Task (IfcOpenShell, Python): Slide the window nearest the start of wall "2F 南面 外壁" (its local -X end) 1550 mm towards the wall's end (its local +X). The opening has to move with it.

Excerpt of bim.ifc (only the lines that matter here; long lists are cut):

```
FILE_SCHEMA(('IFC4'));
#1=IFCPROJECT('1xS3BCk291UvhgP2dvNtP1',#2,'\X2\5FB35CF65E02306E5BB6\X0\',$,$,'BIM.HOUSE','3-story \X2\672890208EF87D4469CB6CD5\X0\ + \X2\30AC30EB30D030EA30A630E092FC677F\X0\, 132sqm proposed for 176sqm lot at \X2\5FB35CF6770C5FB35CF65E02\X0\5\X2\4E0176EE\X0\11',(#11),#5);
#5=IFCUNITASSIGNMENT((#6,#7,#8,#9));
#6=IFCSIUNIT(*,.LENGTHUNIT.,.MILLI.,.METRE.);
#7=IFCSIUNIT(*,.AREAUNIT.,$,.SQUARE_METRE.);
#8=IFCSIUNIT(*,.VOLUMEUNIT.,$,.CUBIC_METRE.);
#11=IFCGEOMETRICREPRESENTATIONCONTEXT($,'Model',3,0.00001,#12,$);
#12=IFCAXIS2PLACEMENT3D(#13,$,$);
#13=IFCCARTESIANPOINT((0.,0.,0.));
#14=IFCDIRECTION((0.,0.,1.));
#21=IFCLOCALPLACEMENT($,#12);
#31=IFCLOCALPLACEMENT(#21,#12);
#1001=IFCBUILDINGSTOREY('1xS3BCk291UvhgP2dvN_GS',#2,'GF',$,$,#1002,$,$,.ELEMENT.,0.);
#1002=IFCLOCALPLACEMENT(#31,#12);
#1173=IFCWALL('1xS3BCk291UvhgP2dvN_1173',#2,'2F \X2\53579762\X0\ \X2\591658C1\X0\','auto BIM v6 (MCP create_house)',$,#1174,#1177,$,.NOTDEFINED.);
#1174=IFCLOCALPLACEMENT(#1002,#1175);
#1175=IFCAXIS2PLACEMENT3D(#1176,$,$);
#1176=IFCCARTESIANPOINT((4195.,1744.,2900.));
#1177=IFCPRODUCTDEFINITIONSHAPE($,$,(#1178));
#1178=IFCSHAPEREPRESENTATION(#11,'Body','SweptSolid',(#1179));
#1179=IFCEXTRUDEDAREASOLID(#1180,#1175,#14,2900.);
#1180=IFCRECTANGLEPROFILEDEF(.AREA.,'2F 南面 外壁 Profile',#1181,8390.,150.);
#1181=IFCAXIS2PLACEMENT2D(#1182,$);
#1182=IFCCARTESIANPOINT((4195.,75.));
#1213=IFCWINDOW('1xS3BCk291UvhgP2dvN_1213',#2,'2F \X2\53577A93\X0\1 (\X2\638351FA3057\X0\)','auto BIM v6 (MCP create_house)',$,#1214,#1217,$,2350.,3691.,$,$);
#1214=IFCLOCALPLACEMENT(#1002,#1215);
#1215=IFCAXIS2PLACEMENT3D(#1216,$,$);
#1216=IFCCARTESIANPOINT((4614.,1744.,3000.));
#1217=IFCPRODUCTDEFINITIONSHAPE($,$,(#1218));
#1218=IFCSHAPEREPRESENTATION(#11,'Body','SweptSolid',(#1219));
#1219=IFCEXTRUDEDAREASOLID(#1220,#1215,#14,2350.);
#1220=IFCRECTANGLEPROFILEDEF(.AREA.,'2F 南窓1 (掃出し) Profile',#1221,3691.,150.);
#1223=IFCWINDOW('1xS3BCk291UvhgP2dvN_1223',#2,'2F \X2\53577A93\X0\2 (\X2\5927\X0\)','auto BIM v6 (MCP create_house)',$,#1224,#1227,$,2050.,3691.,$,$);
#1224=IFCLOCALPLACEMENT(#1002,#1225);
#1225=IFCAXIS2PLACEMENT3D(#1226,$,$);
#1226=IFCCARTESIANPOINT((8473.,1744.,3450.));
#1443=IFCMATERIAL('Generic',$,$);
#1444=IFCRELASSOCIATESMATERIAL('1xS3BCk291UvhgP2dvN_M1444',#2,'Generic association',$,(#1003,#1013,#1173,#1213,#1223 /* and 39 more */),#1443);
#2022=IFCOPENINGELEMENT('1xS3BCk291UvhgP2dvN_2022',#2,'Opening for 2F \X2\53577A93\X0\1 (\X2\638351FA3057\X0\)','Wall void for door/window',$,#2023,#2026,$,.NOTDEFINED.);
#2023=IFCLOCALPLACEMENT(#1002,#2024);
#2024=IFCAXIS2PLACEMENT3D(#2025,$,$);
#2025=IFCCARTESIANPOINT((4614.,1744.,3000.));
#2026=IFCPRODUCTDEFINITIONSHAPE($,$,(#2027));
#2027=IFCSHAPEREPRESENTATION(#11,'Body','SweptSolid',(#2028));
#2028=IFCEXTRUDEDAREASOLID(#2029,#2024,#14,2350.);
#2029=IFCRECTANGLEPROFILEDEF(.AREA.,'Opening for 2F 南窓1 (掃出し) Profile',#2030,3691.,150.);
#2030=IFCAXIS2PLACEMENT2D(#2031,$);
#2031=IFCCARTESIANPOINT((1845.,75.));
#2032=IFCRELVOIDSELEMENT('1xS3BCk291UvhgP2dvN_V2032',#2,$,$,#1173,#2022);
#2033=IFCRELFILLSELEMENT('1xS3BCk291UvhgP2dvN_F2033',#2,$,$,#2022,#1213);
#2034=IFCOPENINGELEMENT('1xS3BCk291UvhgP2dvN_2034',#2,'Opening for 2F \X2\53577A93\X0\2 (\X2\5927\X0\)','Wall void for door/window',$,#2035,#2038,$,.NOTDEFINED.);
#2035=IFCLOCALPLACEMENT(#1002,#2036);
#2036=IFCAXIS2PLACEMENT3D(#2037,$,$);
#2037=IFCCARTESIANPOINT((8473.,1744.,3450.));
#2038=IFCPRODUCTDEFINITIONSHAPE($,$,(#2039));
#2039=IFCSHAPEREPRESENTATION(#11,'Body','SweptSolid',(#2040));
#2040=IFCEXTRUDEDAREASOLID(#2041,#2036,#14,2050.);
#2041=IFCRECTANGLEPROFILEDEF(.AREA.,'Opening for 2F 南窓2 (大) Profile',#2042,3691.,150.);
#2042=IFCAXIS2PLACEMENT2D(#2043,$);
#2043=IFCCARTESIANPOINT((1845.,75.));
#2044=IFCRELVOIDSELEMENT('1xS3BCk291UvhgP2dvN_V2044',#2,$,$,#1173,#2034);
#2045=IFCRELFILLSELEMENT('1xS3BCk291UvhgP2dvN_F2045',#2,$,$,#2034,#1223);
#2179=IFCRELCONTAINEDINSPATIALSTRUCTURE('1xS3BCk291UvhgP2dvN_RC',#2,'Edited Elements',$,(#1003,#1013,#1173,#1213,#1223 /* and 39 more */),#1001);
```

```python
import ifcopenshell
import ifcopenshell.api.geometry
import ifcopenshell.util.placement

model = ifcopenshell.open("bim.ifc")

window = model.by_guid("1xS3BCk291UvhgP2dvN_1213")
opening = window.FillsVoids[0].RelatingOpeningElement
wall = opening.VoidsElements[0].RelatingBuildingElement

wall_matrix = ifcopenshell.util.placement.get_local_placement(wall.ObjectPlacement)
shift = wall_matrix[:3, 0] * 1550.0
before = ifcopenshell.util.placement.get_local_placement(window.ObjectPlacement)[:3, 3].copy()

# The window is not placed relative to its opening, so move both.
for product in (opening, window):
    matrix = ifcopenshell.util.placement.get_local_placement(product.ObjectPlacement)
    matrix[:3, 3] += shift
    ifcopenshell.api.geometry.edit_object_placement(model, product=product, matrix=matrix, is_si=False)

after = ifcopenshell.util.placement.get_local_placement(window.ObjectPlacement)[:3, 3]
print("window moved by", (after - before).round(3) + 0.0)

model.write("bim_v2.ifc")
```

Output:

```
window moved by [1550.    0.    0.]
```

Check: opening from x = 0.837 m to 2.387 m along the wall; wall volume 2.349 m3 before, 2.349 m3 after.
